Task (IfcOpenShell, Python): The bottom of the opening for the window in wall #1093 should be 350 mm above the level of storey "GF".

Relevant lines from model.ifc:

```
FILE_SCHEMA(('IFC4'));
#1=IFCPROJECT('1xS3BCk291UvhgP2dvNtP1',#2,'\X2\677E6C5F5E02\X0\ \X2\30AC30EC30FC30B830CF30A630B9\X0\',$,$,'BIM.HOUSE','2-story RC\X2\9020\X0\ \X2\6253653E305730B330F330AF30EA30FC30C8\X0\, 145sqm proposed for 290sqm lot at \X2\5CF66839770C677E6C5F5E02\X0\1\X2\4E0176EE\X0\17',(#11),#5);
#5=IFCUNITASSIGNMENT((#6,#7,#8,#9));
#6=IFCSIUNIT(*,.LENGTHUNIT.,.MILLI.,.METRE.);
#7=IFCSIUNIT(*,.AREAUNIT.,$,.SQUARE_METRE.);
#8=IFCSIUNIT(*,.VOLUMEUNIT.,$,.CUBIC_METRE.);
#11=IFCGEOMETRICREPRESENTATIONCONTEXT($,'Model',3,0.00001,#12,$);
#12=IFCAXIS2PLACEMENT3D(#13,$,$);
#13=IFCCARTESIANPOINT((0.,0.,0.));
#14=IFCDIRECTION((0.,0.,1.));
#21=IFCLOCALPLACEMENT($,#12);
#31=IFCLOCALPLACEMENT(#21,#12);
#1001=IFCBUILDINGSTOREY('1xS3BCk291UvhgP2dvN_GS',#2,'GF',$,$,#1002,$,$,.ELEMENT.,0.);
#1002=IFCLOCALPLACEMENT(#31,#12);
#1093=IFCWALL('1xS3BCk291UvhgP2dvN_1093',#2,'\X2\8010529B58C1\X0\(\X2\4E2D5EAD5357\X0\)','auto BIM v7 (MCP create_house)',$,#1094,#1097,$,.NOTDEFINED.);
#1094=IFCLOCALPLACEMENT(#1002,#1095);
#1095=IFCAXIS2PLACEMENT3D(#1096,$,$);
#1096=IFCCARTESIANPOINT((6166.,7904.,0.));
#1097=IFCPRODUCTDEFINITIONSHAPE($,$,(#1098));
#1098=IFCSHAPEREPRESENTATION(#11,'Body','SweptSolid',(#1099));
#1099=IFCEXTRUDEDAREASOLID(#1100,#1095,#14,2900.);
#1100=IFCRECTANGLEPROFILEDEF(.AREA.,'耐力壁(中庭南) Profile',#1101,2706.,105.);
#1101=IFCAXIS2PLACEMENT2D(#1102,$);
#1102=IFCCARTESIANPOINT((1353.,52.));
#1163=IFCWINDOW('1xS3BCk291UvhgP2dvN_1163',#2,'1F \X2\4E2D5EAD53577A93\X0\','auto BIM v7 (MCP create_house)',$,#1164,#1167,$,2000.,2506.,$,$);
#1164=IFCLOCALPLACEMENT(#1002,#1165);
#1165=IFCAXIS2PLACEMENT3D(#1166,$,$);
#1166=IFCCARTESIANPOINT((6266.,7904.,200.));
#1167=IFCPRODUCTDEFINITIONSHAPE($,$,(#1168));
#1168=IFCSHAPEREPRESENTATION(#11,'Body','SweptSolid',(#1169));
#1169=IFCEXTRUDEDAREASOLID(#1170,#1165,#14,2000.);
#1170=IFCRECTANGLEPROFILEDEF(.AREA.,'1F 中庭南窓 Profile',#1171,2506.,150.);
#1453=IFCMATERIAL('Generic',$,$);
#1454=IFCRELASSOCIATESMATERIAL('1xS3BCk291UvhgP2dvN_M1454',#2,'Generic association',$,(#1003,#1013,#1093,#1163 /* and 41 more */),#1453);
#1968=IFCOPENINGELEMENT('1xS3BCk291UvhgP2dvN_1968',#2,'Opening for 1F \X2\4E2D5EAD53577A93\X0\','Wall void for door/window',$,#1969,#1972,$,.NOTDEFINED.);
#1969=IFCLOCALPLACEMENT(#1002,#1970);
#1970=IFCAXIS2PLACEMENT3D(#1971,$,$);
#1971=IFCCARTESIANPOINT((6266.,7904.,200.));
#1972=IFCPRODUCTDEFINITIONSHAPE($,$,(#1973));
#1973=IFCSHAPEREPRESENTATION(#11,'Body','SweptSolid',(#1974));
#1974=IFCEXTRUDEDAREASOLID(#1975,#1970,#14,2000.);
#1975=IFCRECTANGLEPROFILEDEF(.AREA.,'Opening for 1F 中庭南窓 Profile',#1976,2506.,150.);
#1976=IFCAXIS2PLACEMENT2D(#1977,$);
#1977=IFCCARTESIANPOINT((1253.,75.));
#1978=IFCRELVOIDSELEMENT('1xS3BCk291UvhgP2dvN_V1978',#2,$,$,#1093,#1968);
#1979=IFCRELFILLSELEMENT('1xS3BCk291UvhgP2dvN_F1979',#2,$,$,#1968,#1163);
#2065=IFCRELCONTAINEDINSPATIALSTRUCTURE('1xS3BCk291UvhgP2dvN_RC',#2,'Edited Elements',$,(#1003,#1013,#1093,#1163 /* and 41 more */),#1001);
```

```python
import numpy as np
import ifcopenshell
import ifcopenshell.api.geometry
import ifcopenshell.geom
import ifcopenshell.util.element
import ifcopenshell.util.placement
import ifcopenshell.util.shape
import ifcopenshell.util.unit

model = ifcopenshell.open("model.ifc")
unit_scale = ifcopenshell.util.unit.calculate_unit_scale(model)

window = model.by_guid("1xS3BCk291UvhgP2dvN_1163")
opening = window.FillsVoids[0].RelatingOpeningElement
storey = ifcopenshell.util.element.get_container(window, ifc_class="IfcBuildingStorey")
level = ifcopenshell.util.placement.get_local_placement(storey.ObjectPlacement)[2, 3]

# The opening's origin need not be at the sill, so measure its lowest point.
shape = ifcopenshell.geom.create_shape(ifcopenshell.geom.settings(), opening)
bottom = ifcopenshell.util.shape.get_shape_bottom_elevation(shape, shape.geometry) / unit_scale
dz = level + 0.35 / unit_scale - bottom

shift = np.array([0.0, 0.0, dz])
# The window is not placed relative to its opening, so move both.
for product in (opening, window):
    matrix = ifcopenshell.util.placement.get_local_placement(product.ObjectPlacement)
    matrix[:3, 3] += shift
    ifcopenshell.api.geometry.edit_object_placement(model, product=product, matrix=matrix, is_si=False)

print(f"moved by {dz * unit_scale:+.3f} m")

model.write("model_rev.ifc")
```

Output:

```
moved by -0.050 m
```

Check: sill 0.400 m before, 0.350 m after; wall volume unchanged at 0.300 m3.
